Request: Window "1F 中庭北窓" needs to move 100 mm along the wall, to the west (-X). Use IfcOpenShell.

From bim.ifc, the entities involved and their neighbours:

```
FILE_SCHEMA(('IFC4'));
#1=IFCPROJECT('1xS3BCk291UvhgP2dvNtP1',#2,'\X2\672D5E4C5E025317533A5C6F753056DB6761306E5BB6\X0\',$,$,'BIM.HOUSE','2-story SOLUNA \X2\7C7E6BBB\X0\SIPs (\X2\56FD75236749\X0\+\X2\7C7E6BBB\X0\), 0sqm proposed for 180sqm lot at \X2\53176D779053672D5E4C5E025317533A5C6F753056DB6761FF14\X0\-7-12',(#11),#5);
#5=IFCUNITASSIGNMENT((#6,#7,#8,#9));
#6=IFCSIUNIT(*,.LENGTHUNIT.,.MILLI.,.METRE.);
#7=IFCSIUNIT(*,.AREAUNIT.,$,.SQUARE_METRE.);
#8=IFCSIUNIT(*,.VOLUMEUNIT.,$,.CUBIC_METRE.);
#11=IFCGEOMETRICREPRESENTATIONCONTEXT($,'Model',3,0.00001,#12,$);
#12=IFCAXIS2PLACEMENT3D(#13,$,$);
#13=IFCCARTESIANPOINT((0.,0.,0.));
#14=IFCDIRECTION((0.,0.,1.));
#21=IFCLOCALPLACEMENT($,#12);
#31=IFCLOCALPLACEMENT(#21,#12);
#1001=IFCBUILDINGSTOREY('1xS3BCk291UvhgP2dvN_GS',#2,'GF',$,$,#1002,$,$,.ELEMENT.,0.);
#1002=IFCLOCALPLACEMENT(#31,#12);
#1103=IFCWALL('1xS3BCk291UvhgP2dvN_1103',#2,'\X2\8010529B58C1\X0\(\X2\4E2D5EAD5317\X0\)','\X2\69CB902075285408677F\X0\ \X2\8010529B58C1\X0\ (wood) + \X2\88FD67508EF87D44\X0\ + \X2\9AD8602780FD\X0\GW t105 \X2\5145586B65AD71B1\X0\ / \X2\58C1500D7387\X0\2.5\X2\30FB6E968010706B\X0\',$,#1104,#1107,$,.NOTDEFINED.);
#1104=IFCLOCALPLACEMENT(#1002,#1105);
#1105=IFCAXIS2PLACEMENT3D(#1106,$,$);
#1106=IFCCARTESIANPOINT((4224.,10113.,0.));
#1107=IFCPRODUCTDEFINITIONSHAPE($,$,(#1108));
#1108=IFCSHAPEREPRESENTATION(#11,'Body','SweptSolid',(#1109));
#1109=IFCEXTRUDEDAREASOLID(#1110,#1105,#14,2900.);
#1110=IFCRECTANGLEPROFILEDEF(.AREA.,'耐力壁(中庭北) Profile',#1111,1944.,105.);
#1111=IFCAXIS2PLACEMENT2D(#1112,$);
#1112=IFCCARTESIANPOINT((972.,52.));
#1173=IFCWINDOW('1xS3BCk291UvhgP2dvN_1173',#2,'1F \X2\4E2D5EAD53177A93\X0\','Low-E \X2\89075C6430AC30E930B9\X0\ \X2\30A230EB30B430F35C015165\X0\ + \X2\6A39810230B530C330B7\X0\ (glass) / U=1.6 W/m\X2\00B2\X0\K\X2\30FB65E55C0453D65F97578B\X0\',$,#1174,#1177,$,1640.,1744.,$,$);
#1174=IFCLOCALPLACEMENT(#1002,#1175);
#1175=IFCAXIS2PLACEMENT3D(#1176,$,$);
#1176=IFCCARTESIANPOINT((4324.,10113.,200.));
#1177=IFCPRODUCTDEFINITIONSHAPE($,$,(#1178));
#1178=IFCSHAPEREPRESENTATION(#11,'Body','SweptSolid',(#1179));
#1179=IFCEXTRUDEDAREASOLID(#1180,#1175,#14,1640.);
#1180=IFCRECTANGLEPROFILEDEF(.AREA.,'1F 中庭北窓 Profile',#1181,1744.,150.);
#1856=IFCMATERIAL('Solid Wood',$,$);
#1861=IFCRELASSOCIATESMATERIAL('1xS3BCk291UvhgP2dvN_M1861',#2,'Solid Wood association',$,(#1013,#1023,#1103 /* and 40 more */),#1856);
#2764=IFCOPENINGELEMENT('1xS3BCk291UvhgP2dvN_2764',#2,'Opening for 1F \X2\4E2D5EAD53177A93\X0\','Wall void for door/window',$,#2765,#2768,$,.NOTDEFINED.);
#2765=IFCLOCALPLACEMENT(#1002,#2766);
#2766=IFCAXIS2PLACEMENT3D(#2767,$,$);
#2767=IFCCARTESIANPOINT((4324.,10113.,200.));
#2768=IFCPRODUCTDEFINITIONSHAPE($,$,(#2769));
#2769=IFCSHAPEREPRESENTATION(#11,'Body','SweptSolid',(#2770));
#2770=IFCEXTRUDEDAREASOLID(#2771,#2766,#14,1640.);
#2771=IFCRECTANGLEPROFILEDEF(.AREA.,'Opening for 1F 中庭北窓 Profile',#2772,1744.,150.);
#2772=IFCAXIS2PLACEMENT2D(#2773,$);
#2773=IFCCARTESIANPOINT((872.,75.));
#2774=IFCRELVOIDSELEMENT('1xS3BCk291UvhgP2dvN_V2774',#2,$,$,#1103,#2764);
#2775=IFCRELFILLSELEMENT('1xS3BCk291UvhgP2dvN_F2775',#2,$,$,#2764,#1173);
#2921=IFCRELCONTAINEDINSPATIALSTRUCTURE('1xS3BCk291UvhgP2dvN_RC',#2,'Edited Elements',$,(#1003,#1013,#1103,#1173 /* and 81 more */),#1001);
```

```python
import ifcopenshell
import ifcopenshell.api.geometry
import ifcopenshell.util.placement
import ifcopenshell.util.unit

model = ifcopenshell.open("bim.ifc")
unit_scale = ifcopenshell.util.unit.calculate_unit_scale(model)

window = model.by_guid("1xS3BCk291UvhgP2dvN_1173")
opening = window.FillsVoids[0].RelatingOpeningElement
wall = opening.VoidsElements[0].RelatingBuildingElement

wall_matrix = ifcopenshell.util.placement.get_local_placement(wall.ObjectPlacement)
shift = wall_matrix[:3, 0] * -0.1 / unit_scale
before = ifcopenshell.util.placement.get_local_placement(window.ObjectPlacement)[:3, 3].copy()

# The window is not placed relative to its opening, so move both.
for product in (opening, window):
    matrix = ifcopenshell.util.placement.get_local_placement(product.ObjectPlacement)
    matrix[:3, 3] += shift
    ifcopenshell.api.geometry.edit_object_placement(model, product=product, matrix=matrix, is_si=False)

after = ifcopenshell.util.placement.get_local_placement(window.ObjectPlacement)[:3, 3]
print("window moved by", (after - before).round(3) + 0.0)

model.write("bim-out.ifc")
```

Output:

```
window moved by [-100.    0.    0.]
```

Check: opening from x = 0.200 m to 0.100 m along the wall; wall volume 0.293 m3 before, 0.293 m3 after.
